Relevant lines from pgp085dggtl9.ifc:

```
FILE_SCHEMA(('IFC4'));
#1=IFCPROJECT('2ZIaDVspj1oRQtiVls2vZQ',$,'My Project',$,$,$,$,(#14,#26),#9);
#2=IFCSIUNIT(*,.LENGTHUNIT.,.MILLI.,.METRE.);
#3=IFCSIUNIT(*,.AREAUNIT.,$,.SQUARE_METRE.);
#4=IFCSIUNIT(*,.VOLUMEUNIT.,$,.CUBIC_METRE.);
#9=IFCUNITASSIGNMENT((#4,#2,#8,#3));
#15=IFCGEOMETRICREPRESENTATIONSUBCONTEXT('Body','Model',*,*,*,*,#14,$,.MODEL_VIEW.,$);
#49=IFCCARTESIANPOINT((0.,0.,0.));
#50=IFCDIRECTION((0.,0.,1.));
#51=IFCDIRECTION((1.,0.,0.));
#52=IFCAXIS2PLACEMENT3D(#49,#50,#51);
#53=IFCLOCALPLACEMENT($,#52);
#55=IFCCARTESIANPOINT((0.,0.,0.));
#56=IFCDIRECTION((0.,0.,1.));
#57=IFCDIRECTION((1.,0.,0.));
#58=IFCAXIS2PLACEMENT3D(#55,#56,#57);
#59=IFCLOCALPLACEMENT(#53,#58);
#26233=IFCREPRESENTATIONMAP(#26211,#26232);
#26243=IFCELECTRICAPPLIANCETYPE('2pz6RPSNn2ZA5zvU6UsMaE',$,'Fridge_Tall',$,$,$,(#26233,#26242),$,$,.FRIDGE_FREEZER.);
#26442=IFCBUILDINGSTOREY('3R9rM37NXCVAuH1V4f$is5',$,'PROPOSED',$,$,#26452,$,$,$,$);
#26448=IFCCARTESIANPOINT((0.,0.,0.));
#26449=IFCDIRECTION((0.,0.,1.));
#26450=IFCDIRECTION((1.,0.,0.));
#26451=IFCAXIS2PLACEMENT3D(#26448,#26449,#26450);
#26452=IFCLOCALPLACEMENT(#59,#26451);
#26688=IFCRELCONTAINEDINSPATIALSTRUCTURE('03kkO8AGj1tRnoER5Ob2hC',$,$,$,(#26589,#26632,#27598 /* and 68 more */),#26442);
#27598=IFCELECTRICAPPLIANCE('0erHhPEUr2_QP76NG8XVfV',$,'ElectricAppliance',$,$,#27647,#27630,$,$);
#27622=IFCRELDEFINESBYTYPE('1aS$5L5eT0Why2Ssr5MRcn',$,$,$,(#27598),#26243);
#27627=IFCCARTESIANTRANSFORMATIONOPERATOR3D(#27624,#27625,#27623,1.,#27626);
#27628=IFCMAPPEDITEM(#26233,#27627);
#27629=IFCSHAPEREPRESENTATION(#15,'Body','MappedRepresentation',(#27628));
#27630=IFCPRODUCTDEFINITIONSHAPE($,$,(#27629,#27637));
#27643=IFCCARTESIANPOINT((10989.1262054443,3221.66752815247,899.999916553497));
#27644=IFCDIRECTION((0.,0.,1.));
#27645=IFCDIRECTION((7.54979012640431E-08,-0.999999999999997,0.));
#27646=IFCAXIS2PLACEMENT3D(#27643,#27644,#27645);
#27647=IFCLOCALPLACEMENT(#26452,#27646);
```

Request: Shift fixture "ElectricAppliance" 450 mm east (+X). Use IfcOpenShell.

```python
import ifcopenshell
import ifcopenshell.api.geometry
import ifcopenshell.util.placement

model = ifcopenshell.open("pgp085dggtl9.ifc")

item = model.by_guid("0erHhPEUr2_QP76NG8XVfV")
matrix = ifcopenshell.util.placement.get_local_placement(item.ObjectPlacement)
matrix[0, 3] += 450.0
ifcopenshell.api.geometry.edit_object_placement(model, product=item, matrix=matrix, is_si=False)

print(ifcopenshell.util.placement.get_local_placement(item.ObjectPlacement).round(3) + 0.0)

model.write("pgp085dggtl9_v2.ifc")
```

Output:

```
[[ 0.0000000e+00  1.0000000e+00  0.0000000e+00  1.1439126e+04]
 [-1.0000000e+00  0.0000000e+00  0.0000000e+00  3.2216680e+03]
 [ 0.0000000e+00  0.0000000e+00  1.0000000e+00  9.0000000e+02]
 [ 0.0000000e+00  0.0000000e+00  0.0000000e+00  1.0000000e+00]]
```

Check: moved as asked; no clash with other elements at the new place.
